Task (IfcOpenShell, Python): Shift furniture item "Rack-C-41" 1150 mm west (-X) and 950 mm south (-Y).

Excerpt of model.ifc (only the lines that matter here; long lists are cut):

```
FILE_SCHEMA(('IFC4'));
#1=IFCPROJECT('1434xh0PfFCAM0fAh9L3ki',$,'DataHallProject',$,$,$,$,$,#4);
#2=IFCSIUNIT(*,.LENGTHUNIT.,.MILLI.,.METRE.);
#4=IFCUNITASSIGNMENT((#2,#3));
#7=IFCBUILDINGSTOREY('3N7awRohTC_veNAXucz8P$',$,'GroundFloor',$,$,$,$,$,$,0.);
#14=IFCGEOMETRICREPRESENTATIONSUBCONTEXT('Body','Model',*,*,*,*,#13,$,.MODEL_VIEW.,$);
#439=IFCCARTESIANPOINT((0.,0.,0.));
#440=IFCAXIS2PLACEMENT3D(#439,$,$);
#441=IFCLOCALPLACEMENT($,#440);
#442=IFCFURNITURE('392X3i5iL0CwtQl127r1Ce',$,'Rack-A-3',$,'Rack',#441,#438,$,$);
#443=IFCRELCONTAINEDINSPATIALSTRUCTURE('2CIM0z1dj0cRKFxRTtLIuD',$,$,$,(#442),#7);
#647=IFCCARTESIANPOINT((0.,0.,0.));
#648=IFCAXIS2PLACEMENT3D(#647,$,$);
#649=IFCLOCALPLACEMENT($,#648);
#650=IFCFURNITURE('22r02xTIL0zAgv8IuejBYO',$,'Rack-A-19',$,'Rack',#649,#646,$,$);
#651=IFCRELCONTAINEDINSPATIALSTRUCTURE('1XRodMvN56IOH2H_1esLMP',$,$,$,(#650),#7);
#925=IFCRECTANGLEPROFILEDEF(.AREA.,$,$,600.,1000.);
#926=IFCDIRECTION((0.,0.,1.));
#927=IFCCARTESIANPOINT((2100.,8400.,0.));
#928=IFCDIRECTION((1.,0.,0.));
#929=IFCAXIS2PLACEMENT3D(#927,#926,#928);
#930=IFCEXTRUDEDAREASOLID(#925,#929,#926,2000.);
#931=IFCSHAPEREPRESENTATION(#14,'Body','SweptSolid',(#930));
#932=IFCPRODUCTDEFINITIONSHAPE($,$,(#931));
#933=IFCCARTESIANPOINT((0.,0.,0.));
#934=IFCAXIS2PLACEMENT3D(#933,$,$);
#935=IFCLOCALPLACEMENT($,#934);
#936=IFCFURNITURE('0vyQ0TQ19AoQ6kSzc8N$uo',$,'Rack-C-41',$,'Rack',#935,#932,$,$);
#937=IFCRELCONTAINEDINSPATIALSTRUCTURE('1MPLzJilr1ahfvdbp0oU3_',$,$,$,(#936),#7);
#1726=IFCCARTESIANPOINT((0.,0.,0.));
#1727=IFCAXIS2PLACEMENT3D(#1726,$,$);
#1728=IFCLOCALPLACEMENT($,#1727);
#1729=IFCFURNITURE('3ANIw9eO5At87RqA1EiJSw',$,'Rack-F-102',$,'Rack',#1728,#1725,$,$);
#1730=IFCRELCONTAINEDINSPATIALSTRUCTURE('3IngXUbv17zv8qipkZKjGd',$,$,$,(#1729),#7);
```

```python
import ifcopenshell
import ifcopenshell.api.geometry
import ifcopenshell.util.placement
import ifcopenshell.util.unit

model = ifcopenshell.open("model.ifc")
unit_scale = ifcopenshell.util.unit.calculate_unit_scale(model)

item = model.by_guid("0vyQ0TQ19AoQ6kSzc8N$uo")
matrix = ifcopenshell.util.placement.get_local_placement(item.ObjectPlacement)
matrix[0, 3] -= 1.15 / unit_scale
matrix[1, 3] -= 0.95 / unit_scale
ifcopenshell.api.geometry.edit_object_placement(model, product=item, matrix=matrix, is_si=False)

print(ifcopenshell.util.placement.get_local_placement(item.ObjectPlacement).round(3) + 0.0)

model.write("model_edited.ifc")
```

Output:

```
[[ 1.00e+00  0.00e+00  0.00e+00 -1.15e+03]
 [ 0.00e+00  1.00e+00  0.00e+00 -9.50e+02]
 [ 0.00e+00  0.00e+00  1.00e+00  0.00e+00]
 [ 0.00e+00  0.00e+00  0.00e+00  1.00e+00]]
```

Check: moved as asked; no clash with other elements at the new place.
